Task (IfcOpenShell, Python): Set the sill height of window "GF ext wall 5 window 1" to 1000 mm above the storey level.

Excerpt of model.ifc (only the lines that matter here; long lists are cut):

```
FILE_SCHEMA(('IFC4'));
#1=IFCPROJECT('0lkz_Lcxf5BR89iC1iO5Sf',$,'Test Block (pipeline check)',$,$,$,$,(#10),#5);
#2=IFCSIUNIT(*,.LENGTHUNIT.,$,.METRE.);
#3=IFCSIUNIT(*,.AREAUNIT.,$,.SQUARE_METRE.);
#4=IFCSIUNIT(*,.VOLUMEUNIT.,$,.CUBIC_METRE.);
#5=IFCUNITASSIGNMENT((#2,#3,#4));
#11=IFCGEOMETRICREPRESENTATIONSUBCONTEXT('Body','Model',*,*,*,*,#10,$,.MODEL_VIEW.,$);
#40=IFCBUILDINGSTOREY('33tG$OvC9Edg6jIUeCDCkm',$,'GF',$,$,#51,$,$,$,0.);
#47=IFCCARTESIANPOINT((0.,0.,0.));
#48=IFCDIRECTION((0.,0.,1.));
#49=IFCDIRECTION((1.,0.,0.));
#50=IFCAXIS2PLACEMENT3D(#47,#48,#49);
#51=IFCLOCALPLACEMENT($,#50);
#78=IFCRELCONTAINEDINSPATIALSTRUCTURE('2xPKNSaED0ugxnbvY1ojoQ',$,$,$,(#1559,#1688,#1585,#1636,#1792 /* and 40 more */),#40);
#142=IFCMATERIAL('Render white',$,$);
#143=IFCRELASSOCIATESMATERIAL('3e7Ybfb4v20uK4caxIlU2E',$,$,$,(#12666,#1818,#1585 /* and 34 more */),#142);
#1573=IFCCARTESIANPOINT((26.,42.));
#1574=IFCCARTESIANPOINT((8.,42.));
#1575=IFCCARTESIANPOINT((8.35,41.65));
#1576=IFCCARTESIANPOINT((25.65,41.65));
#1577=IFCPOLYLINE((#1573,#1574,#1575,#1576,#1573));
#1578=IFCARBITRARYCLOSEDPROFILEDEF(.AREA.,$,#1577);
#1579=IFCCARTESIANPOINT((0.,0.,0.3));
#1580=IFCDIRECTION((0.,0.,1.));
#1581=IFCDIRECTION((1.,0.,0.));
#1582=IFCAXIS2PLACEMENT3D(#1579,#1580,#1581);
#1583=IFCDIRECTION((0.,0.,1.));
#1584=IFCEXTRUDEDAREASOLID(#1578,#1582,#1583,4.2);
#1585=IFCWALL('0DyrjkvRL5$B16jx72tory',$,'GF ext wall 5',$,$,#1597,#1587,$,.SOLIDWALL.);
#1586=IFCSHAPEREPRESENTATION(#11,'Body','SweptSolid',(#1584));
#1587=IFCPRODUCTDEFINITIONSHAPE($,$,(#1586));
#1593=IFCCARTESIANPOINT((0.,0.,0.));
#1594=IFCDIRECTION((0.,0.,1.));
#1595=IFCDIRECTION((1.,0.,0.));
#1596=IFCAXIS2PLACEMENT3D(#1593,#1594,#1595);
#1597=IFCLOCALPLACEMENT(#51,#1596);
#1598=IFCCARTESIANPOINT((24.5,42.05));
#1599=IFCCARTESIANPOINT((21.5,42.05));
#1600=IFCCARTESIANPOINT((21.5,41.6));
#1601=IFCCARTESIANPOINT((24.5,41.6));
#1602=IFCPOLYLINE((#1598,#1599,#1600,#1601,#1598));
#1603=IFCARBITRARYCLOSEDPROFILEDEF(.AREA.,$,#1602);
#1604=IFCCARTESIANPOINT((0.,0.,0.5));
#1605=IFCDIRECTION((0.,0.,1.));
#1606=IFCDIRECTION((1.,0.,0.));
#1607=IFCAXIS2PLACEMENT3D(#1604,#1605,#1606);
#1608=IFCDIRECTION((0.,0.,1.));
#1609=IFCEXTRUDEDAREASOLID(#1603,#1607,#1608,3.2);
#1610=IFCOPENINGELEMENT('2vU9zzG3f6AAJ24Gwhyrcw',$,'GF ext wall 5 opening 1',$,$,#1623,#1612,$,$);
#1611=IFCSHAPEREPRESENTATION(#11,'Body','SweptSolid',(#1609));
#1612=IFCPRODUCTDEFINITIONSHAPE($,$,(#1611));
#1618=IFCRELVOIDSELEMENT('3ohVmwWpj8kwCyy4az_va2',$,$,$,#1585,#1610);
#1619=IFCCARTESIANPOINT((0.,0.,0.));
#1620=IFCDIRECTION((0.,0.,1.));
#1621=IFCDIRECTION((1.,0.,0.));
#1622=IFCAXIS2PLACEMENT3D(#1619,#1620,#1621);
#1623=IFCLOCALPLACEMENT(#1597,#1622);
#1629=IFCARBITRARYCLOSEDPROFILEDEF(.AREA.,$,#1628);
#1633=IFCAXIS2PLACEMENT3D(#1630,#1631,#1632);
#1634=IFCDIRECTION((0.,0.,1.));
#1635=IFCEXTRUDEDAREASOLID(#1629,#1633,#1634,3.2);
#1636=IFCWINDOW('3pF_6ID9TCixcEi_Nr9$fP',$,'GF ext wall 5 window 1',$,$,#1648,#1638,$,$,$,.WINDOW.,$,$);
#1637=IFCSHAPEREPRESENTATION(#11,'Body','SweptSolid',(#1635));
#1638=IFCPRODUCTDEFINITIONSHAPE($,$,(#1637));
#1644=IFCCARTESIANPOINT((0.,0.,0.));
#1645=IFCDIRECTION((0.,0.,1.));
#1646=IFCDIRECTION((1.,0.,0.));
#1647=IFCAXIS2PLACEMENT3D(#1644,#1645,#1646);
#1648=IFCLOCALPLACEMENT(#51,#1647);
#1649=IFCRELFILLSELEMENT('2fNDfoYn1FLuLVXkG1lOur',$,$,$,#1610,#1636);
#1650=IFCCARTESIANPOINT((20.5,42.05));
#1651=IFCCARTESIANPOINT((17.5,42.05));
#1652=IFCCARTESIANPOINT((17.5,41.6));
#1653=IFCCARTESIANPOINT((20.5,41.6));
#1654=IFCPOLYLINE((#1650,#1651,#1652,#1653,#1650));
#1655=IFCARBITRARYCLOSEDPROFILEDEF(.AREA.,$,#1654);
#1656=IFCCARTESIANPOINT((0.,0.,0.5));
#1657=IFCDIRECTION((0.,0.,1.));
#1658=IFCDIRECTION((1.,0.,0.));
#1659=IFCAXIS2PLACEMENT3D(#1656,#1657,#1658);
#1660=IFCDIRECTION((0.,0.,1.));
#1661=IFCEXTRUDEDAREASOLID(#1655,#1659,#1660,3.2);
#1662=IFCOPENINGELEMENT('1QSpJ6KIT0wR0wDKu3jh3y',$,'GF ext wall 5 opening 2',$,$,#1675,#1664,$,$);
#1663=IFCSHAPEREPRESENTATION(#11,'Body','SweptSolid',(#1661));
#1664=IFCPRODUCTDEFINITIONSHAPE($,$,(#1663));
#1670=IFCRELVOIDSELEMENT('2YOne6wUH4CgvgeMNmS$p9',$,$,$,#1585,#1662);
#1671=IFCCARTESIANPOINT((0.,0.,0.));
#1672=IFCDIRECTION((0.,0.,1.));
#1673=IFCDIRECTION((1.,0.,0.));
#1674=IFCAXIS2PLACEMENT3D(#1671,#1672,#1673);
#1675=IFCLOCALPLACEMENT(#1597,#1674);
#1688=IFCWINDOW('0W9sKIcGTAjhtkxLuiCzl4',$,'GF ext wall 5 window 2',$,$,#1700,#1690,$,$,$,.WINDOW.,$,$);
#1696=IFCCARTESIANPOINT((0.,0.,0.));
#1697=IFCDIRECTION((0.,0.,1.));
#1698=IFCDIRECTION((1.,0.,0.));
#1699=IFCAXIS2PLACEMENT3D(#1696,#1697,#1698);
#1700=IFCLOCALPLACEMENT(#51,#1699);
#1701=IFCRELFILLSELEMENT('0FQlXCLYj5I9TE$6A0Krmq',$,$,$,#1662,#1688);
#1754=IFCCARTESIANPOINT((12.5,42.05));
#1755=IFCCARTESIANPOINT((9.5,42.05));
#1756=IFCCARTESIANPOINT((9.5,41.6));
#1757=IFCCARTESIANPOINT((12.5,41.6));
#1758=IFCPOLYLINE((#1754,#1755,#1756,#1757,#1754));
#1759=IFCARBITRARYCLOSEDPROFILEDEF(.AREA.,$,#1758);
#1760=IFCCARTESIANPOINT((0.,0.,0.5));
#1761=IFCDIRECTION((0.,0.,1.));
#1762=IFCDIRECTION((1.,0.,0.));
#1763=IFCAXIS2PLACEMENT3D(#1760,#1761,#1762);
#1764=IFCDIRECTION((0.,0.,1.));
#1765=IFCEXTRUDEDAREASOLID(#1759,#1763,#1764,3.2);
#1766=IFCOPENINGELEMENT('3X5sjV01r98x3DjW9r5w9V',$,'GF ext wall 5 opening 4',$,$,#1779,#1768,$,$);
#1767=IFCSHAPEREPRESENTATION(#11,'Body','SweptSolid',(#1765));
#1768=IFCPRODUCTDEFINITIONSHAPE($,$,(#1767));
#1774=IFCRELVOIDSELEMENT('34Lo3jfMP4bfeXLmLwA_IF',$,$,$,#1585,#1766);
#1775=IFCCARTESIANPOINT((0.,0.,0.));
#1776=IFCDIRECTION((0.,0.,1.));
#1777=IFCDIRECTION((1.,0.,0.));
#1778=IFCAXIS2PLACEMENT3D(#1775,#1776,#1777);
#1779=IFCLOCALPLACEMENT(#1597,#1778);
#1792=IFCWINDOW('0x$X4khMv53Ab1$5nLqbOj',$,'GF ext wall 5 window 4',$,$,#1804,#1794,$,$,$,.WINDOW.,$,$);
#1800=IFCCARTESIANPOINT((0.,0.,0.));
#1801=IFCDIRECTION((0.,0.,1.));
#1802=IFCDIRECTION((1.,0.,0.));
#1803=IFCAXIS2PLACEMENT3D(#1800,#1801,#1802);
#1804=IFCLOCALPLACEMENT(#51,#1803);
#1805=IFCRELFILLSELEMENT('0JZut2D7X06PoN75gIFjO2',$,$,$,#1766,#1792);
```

```python
import numpy as np
import ifcopenshell
import ifcopenshell.api.geometry
import ifcopenshell.geom
import ifcopenshell.util.element
import ifcopenshell.util.placement
import ifcopenshell.util.shape
import ifcopenshell.util.unit

model = ifcopenshell.open("model.ifc")
unit_scale = ifcopenshell.util.unit.calculate_unit_scale(model)

window = model.by_guid("3pF_6ID9TCixcEi_Nr9$fP")
opening = window.FillsVoids[0].RelatingOpeningElement
storey = ifcopenshell.util.element.get_container(window, ifc_class="IfcBuildingStorey")
level = ifcopenshell.util.placement.get_local_placement(storey.ObjectPlacement)[2, 3]

# The opening's origin need not be at the sill, so measure its lowest point.
shape = ifcopenshell.geom.create_shape(ifcopenshell.geom.settings(), opening)
bottom = ifcopenshell.util.shape.get_shape_bottom_elevation(shape, shape.geometry) / unit_scale
dz = level + 1 / unit_scale - bottom

shift = np.array([0.0, 0.0, dz])
# The window is not placed relative to its opening, so move both.
for product in (opening, window):
    matrix = ifcopenshell.util.placement.get_local_placement(product.ObjectPlacement)
    matrix[:3, 3] += shift
    ifcopenshell.api.geometry.edit_object_placement(model, product=product, matrix=matrix, is_si=False)

print(f"moved by {dz * unit_scale:+.3f} m")

model.write("model-out.ifc")
```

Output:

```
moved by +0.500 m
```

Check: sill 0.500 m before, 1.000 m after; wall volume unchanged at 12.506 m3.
